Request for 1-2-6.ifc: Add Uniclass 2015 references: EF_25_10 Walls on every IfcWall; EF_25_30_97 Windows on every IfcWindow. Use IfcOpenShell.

First a look at what the model holds.

```python
import ifcopenshell

model = ifcopenshell.open("1-2-6.ifc")
print(model.schema)
print("classifications:", [c.Name for c in model.by_type("IfcClassification")])
for ifc_class in ("IfcDoor", "IfcRoof", "IfcStair", "IfcWall", "IfcWindow"):
    print(ifc_class, len(model.by_type(ifc_class)))
```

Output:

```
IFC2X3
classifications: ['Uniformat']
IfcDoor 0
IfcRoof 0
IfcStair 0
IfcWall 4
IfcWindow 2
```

```python
import ifcopenshell
import ifcopenshell.api.classification

model = ifcopenshell.open("1-2-6.ifc")

# IFC2X3 requires Source and Edition and has no link from the project to the system.
system = model.create_entity("IfcClassification", Source="NBS", Edition="2015", Name="Uniclass 2015")

codes = {
    "IfcWall": ("EF_25_10", "Walls"),
    "IfcWindow": ("EF_25_30_97", "Windows"),
}
for ifc_class, (code, name) in codes.items():
    products = model.by_type(ifc_class)
    ifcopenshell.api.classification.add_reference(
        model, products=products, classification=system, identification=code, name=name
    )
    print(code, len(products))

model.write("1-2-6_v2.ifc")
```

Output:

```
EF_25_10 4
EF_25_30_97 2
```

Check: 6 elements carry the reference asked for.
